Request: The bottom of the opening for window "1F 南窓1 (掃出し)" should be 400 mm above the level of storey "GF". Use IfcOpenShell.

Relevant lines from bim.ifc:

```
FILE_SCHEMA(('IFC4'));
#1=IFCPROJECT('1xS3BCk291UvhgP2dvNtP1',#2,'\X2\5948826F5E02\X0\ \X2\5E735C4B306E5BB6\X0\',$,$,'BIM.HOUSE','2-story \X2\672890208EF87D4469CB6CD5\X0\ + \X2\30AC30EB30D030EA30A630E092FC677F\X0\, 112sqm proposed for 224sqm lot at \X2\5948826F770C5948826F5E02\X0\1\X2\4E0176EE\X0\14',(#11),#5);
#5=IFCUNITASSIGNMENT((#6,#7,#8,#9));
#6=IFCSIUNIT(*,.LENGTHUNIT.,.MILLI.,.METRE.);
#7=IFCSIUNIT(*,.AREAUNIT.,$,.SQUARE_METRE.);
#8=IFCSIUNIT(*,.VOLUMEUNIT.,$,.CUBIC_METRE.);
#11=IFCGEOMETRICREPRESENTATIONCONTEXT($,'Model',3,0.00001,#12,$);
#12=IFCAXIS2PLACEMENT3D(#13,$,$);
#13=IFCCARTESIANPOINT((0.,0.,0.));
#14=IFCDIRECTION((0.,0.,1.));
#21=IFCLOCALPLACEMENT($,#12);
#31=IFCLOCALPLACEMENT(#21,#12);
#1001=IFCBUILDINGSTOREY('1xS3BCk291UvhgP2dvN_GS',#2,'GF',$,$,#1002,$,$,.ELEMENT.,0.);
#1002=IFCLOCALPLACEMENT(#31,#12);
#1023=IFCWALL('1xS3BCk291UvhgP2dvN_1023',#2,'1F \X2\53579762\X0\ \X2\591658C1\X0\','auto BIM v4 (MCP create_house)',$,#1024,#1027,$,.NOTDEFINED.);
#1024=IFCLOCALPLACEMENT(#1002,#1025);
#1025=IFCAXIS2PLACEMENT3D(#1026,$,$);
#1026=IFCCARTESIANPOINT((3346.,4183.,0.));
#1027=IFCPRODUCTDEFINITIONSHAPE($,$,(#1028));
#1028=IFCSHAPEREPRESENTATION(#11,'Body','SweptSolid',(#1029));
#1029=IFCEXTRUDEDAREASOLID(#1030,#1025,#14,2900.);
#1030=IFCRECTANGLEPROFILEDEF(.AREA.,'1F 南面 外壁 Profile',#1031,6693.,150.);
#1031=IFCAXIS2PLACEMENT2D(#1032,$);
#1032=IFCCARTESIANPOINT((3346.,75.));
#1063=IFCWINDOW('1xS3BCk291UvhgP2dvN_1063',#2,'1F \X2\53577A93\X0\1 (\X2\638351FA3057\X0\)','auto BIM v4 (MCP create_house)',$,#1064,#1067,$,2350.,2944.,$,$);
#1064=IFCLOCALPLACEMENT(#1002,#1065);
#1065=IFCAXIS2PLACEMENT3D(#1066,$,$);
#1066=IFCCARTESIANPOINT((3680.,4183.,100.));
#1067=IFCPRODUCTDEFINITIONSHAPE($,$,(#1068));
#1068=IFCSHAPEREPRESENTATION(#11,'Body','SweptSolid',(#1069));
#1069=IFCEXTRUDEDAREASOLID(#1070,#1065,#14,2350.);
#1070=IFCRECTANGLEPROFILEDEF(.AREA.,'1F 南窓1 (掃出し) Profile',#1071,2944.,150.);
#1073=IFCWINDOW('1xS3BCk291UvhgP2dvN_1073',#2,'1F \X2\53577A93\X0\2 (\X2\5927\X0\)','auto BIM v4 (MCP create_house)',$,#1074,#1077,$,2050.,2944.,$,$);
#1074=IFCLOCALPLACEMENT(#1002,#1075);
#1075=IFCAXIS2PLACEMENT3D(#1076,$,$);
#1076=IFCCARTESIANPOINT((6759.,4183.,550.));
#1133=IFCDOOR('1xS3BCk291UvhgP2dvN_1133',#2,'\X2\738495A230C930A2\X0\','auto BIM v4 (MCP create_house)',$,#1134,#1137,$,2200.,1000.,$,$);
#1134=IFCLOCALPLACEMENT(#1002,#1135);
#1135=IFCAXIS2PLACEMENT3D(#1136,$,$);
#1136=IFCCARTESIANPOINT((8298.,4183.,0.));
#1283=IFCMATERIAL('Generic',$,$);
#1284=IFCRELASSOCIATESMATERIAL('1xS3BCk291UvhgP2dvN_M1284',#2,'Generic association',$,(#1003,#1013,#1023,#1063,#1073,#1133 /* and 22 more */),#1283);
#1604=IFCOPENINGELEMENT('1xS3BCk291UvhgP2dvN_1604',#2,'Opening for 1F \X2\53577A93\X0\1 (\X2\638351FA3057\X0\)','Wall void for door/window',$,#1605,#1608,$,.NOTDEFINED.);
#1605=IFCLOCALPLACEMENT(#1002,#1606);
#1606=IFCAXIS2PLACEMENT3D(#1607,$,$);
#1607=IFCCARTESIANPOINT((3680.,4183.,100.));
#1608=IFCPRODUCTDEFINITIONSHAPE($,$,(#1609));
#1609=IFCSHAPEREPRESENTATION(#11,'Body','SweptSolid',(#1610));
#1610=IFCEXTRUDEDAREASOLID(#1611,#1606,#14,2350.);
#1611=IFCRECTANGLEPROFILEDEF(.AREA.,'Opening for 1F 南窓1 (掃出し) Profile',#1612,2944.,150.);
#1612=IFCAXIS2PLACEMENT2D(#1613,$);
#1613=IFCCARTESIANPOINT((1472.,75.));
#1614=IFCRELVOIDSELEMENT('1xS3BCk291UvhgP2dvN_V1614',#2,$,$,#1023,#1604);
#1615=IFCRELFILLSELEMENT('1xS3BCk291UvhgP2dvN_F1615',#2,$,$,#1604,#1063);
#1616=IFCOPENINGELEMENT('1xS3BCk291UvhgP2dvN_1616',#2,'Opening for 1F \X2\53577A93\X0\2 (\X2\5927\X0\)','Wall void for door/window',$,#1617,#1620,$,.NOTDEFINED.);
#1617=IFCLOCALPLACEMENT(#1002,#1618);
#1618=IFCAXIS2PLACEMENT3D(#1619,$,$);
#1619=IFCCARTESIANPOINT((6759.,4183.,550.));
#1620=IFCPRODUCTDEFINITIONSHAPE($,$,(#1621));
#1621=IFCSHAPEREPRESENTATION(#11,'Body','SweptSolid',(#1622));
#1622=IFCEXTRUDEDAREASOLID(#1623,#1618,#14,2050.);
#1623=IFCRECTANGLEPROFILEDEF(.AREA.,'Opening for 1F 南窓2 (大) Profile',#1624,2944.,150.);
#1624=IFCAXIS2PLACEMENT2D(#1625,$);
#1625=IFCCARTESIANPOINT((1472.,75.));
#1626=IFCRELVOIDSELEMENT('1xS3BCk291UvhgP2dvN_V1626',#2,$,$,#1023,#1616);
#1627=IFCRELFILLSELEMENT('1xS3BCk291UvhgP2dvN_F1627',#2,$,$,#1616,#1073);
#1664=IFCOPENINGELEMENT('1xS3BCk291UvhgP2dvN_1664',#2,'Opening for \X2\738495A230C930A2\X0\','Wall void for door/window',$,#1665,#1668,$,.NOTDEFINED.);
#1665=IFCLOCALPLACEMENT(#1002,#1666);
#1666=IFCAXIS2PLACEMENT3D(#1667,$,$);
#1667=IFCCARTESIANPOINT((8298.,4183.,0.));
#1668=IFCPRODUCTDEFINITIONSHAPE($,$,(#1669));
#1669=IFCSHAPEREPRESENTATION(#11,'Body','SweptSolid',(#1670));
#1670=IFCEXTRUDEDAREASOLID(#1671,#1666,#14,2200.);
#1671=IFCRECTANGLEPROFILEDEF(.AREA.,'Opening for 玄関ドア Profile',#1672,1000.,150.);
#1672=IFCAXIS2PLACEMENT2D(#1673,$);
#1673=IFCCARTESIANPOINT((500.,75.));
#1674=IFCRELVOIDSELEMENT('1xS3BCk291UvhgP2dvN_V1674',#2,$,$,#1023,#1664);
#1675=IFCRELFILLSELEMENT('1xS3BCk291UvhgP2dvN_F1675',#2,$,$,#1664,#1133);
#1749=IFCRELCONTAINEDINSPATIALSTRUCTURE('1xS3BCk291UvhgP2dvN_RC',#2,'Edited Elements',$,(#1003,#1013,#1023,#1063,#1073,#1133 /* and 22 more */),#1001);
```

```python
import numpy as np
import ifcopenshell
import ifcopenshell.api.geometry
import ifcopenshell.geom
import ifcopenshell.util.element
import ifcopenshell.util.placement
import ifcopenshell.util.shape
import ifcopenshell.util.unit

model = ifcopenshell.open("bim.ifc")
unit_scale = ifcopenshell.util.unit.calculate_unit_scale(model)

window = model.by_id(1063)
opening = window.FillsVoids[0].RelatingOpeningElement
storey = ifcopenshell.util.element.get_container(window, ifc_class="IfcBuildingStorey")
level = ifcopenshell.util.placement.get_local_placement(storey.ObjectPlacement)[2, 3]

# The opening's origin need not be at the sill, so measure its lowest point.
shape = ifcopenshell.geom.create_shape(ifcopenshell.geom.settings(), opening)
bottom = ifcopenshell.util.shape.get_shape_bottom_elevation(shape, shape.geometry) / unit_scale
dz = level + 0.4 / unit_scale - bottom

shift = np.array([0.0, 0.0, dz])
# The window is not placed relative to its opening, so move both.
for product in (opening, window):
    matrix = ifcopenshell.util.placement.get_local_placement(product.ObjectPlacement)
    matrix[:3, 3] += shift
    ifcopenshell.api.geometry.edit_object_placement(model, product=product, matrix=matrix, is_si=False)

print(f"moved by {dz * unit_scale:+.3f} m")

model.write("bim_rev.ifc")
```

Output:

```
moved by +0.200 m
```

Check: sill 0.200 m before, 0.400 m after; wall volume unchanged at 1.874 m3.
